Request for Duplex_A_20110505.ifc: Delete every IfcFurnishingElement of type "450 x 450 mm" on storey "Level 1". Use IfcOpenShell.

First a look at what the model holds.

```python
import ifcopenshell
import ifcopenshell.util.element

model = ifcopenshell.open("Duplex_A_20110505.ifc")
print(model.schema)
storey = next(s for s in model.by_type("IfcBuildingStorey") if s.Name == "Level 1")
furniture = [e for e in ifcopenshell.util.element.get_decomposition(storey) if e.is_a("IfcFurnishingElement")]
seen = {}
for e in furniture:
    element_type = ifcopenshell.util.element.get_type(e)
    name = element_type.Name if element_type not in (None, e) else None
    seen[name] = seen.get(name, 0) + 1
for name, count in sorted(seen.items(), key=str):
    print(count, "x", name)
```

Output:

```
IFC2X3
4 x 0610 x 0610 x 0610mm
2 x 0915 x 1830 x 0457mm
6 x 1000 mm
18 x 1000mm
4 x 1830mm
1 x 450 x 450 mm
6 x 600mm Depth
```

```python
import ifcopenshell
import ifcopenshell.api.root
import ifcopenshell.util.element

model = ifcopenshell.open("Duplex_A_20110505.ifc")

storey = next(s for s in model.by_type("IfcBuildingStorey") if s.Name == "Level 1")
furniture = [e for e in ifcopenshell.util.element.get_decomposition(storey) if e.is_a("IfcFurnishingElement")]
targets = [e for e in furniture if (t := ifcopenshell.util.element.get_type(e)) not in (None, e) and t.Name == "450 x 450 mm"]

for e in targets:
    ifcopenshell.api.root.remove_product(model, product=e)
print(len(targets), "removed")

model.write("Duplex_A_20110505-out.ifc")
```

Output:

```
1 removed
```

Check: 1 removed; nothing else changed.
